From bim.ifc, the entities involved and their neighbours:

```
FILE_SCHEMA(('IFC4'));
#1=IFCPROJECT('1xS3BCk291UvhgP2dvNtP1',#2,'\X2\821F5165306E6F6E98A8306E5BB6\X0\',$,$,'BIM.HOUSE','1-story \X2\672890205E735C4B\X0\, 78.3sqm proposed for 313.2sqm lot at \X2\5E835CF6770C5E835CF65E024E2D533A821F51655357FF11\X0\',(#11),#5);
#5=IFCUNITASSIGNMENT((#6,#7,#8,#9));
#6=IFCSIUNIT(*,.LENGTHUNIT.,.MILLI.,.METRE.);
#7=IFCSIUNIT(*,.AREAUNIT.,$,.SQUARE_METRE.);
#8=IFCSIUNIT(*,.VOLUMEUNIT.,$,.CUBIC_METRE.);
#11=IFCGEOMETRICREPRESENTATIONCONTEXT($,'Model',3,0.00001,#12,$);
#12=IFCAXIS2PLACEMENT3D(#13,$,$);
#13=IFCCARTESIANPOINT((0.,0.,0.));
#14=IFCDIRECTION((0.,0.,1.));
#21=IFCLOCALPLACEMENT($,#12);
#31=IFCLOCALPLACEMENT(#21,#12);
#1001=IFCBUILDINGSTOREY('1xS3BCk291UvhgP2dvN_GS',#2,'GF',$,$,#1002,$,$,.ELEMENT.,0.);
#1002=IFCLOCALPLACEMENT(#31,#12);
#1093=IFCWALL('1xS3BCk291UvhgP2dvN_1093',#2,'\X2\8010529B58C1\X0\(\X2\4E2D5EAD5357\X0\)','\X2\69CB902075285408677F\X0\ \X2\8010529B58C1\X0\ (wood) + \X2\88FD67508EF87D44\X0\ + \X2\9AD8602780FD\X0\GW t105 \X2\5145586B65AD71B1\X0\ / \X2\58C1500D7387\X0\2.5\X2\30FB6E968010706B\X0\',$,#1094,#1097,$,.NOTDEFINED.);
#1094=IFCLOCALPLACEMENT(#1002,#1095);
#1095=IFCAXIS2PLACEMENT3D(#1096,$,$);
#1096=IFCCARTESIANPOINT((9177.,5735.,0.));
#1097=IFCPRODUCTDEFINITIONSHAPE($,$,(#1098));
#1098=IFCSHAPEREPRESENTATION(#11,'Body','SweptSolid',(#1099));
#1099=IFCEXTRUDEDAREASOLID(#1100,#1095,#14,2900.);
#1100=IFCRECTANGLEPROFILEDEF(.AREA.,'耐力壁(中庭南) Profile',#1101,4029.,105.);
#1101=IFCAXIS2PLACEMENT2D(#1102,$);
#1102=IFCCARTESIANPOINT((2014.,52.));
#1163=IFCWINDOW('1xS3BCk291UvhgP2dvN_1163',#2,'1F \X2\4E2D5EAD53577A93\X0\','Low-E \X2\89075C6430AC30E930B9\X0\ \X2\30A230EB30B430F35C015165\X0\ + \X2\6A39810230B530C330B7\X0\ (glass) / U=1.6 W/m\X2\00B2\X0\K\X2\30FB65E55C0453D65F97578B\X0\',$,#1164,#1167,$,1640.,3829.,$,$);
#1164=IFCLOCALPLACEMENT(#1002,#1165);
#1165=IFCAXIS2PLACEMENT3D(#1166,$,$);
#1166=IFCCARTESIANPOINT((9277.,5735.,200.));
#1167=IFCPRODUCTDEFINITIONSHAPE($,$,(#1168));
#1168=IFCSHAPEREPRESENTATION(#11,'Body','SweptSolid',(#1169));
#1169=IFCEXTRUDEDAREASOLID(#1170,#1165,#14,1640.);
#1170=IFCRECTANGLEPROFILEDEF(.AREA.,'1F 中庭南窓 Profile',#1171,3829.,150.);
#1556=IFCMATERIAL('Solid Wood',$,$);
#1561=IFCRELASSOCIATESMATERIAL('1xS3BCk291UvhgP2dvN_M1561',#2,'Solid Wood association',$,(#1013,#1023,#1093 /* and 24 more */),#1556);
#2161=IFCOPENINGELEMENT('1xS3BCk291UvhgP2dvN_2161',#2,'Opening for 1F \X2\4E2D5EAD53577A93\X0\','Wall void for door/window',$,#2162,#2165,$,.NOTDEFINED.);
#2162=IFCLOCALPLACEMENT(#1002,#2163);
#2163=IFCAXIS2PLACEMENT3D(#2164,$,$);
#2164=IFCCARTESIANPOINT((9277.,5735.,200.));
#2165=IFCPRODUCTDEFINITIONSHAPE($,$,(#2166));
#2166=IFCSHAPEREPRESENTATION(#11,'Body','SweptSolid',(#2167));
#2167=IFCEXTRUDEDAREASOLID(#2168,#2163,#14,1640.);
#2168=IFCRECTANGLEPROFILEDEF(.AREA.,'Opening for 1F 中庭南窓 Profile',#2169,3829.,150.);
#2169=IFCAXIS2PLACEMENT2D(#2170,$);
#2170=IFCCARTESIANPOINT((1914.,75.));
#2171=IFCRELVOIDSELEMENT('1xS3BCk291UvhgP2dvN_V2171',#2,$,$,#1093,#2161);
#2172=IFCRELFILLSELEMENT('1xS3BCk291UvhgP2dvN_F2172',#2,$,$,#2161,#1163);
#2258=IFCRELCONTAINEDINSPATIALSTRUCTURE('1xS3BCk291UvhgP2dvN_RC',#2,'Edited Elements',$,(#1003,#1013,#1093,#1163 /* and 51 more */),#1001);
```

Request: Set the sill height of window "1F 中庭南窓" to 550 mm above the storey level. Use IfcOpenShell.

```python
import numpy as np
import ifcopenshell
import ifcopenshell.api.geometry
import ifcopenshell.geom
import ifcopenshell.util.element
import ifcopenshell.util.placement
import ifcopenshell.util.shape
import ifcopenshell.util.unit

model = ifcopenshell.open("bim.ifc")
unit_scale = ifcopenshell.util.unit.calculate_unit_scale(model)

window = model.by_id(1163)
opening = window.FillsVoids[0].RelatingOpeningElement
storey = ifcopenshell.util.element.get_container(window, ifc_class="IfcBuildingStorey")
level = ifcopenshell.util.placement.get_local_placement(storey.ObjectPlacement)[2, 3]

# The opening's origin need not be at the sill, so measure its lowest point.
shape = ifcopenshell.geom.create_shape(ifcopenshell.geom.settings(), opening)
bottom = ifcopenshell.util.shape.get_shape_bottom_elevation(shape, shape.geometry) / unit_scale
dz = level + 0.55 / unit_scale - bottom

shift = np.array([0.0, 0.0, dz])
# The window is not placed relative to its opening, so move both.
for product in (opening, window):
    matrix = ifcopenshell.util.placement.get_local_placement(product.ObjectPlacement)
    matrix[:3, 3] += shift
    ifcopenshell.api.geometry.edit_object_placement(model, product=product, matrix=matrix, is_si=False)

print(f"moved by {dz * unit_scale:+.3f} m")

model.write("bim-out.ifc")
```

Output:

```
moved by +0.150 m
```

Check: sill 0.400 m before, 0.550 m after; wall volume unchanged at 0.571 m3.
